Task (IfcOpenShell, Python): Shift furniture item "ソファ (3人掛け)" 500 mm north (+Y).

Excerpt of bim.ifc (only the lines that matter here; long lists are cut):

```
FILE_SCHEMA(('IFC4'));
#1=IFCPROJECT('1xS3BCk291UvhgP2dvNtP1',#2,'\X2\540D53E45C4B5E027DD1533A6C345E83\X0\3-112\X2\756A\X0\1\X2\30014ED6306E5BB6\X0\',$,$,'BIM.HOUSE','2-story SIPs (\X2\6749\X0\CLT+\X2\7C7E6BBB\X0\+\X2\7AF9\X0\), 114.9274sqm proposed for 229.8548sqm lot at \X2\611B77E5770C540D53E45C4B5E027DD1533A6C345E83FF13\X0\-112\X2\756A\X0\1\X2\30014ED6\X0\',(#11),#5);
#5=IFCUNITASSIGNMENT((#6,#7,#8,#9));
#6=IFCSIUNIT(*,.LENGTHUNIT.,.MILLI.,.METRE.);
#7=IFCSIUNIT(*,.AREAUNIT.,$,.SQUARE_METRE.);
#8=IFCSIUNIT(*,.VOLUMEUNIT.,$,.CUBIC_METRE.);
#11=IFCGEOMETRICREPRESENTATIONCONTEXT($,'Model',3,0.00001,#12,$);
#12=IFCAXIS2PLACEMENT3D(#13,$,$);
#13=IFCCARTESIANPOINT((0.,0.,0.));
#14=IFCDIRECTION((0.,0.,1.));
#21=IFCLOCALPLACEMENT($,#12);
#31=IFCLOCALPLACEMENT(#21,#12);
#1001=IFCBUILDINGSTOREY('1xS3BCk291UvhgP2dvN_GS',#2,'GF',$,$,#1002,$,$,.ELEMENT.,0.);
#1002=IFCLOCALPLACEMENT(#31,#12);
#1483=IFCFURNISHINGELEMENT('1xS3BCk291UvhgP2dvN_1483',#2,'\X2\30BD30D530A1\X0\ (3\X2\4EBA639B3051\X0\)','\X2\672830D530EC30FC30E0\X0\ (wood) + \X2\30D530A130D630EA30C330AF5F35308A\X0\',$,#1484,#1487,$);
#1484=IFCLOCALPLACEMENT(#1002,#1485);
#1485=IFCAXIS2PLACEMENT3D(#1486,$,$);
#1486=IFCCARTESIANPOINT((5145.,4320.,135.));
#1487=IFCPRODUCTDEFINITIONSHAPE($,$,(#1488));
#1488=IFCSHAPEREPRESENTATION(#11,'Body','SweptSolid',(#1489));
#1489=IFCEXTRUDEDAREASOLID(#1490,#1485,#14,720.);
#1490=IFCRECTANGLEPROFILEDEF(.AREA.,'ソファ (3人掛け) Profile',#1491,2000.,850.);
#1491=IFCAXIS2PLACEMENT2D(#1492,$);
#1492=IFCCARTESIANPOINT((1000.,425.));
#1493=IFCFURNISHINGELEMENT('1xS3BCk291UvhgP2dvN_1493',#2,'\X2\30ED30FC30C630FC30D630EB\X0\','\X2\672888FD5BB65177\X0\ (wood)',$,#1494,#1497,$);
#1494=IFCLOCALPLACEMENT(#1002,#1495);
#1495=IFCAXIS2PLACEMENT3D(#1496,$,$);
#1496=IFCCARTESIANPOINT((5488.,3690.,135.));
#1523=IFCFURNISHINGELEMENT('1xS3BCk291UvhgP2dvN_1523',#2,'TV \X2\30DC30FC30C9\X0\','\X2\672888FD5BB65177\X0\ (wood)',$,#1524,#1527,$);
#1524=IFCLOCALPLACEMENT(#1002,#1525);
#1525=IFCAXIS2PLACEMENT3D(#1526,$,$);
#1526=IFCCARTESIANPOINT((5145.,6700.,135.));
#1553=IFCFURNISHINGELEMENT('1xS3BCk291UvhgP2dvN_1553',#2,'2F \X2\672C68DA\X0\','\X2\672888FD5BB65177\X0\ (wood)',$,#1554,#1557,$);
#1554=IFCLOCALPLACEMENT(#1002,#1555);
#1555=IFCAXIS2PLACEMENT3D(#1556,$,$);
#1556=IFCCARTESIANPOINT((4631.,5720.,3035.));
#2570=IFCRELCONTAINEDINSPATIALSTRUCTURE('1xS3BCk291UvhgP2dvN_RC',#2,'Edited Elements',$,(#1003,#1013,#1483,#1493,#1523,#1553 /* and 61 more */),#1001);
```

```python
import ifcopenshell
import ifcopenshell.api.geometry
import ifcopenshell.util.placement

model = ifcopenshell.open("bim.ifc")

item = model.by_guid("1xS3BCk291UvhgP2dvN_1483")
matrix = ifcopenshell.util.placement.get_local_placement(item.ObjectPlacement)
matrix[1, 3] += 500.0
ifcopenshell.api.geometry.edit_object_placement(model, product=item, matrix=matrix, is_si=False)

print(ifcopenshell.util.placement.get_local_placement(item.ObjectPlacement).round(3) + 0.0)

model.write("bim_v2.ifc")
```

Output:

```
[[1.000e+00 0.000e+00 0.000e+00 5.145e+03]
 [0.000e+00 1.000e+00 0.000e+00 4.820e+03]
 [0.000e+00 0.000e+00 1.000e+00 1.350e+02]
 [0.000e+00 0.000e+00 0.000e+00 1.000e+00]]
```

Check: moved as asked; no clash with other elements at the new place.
